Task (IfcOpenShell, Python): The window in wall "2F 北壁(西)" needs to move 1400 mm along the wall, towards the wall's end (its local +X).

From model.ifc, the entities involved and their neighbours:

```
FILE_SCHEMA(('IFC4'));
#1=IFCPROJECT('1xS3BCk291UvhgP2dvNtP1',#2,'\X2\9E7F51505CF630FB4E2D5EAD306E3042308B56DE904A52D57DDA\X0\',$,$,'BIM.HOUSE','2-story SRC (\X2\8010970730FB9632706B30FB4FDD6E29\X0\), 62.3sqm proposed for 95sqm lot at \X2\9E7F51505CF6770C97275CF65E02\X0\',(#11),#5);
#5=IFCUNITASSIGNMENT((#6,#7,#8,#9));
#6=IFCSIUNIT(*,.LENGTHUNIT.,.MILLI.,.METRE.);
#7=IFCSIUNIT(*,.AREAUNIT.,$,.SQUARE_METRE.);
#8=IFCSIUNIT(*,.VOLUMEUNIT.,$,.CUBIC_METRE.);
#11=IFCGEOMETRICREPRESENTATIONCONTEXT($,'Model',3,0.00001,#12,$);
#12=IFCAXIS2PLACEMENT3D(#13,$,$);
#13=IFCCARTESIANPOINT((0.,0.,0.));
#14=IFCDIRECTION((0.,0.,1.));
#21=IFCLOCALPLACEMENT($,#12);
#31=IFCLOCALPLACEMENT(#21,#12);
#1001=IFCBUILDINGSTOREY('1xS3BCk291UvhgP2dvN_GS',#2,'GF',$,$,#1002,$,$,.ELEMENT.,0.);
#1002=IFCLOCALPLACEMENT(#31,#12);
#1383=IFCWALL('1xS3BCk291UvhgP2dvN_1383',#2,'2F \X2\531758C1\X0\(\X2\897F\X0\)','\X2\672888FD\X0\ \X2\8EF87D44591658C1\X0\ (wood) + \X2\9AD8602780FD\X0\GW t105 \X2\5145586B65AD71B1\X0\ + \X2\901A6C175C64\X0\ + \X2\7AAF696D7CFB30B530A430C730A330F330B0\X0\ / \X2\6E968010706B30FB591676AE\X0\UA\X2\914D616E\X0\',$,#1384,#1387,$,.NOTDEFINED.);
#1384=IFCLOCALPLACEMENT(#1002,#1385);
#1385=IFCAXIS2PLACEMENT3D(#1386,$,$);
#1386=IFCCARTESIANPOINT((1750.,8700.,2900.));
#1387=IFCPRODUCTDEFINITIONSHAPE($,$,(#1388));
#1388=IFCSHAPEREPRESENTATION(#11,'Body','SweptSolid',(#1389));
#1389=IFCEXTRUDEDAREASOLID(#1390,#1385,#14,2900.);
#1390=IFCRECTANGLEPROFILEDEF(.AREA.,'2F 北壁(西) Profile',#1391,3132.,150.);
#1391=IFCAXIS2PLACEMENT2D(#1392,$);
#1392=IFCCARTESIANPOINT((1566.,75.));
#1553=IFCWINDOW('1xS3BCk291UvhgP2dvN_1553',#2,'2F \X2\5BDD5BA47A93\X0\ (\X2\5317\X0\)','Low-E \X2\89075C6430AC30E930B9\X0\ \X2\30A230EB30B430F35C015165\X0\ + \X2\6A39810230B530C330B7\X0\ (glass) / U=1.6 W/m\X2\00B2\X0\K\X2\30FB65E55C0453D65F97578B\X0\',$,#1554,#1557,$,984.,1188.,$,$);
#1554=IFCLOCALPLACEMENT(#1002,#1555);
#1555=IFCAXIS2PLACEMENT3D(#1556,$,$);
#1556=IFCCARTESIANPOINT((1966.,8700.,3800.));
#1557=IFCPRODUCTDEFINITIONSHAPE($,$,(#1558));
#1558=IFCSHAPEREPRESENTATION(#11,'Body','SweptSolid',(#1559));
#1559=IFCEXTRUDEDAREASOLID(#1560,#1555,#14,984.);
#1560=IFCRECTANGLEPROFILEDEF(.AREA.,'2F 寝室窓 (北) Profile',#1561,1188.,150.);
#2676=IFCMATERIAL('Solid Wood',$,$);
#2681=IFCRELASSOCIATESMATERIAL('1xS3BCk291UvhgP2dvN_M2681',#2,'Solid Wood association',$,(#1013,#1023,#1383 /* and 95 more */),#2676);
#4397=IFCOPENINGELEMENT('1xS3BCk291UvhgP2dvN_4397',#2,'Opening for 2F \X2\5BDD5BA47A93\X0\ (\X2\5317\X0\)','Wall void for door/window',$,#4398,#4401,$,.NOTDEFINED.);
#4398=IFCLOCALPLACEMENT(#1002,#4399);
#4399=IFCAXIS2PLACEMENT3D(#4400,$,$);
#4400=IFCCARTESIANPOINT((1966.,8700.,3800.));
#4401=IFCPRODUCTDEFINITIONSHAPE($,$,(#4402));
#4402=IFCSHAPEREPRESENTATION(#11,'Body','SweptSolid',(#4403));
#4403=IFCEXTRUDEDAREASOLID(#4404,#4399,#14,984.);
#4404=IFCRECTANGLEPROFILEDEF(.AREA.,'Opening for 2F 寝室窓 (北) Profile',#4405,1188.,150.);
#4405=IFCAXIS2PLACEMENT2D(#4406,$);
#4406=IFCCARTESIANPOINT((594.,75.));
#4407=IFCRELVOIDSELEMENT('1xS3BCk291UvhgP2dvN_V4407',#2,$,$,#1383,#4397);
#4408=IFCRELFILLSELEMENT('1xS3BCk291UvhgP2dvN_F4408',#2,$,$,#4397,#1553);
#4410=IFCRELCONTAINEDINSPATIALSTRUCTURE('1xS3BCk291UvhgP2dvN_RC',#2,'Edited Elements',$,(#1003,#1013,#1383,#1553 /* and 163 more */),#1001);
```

```python
import ifcopenshell
import ifcopenshell.api.geometry
import ifcopenshell.util.placement

model = ifcopenshell.open("model.ifc")

window = model.by_guid("1xS3BCk291UvhgP2dvN_1553")
opening = window.FillsVoids[0].RelatingOpeningElement
wall = opening.VoidsElements[0].RelatingBuildingElement

wall_matrix = ifcopenshell.util.placement.get_local_placement(wall.ObjectPlacement)
shift = wall_matrix[:3, 0] * 1400.0
before = ifcopenshell.util.placement.get_local_placement(window.ObjectPlacement)[:3, 3].copy()

# The window is not placed relative to its opening, so move both.
for product in (opening, window):
    matrix = ifcopenshell.util.placement.get_local_placement(product.ObjectPlacement)
    matrix[:3, 3] += shift
    ifcopenshell.api.geometry.edit_object_placement(model, product=product, matrix=matrix, is_si=False)

after = ifcopenshell.util.placement.get_local_placement(window.ObjectPlacement)[:3, 3]
print("window moved by", (after - before).round(3) + 0.0)

model.write("model_v2.ifc")
```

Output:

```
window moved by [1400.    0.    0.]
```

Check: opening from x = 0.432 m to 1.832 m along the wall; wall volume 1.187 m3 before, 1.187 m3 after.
